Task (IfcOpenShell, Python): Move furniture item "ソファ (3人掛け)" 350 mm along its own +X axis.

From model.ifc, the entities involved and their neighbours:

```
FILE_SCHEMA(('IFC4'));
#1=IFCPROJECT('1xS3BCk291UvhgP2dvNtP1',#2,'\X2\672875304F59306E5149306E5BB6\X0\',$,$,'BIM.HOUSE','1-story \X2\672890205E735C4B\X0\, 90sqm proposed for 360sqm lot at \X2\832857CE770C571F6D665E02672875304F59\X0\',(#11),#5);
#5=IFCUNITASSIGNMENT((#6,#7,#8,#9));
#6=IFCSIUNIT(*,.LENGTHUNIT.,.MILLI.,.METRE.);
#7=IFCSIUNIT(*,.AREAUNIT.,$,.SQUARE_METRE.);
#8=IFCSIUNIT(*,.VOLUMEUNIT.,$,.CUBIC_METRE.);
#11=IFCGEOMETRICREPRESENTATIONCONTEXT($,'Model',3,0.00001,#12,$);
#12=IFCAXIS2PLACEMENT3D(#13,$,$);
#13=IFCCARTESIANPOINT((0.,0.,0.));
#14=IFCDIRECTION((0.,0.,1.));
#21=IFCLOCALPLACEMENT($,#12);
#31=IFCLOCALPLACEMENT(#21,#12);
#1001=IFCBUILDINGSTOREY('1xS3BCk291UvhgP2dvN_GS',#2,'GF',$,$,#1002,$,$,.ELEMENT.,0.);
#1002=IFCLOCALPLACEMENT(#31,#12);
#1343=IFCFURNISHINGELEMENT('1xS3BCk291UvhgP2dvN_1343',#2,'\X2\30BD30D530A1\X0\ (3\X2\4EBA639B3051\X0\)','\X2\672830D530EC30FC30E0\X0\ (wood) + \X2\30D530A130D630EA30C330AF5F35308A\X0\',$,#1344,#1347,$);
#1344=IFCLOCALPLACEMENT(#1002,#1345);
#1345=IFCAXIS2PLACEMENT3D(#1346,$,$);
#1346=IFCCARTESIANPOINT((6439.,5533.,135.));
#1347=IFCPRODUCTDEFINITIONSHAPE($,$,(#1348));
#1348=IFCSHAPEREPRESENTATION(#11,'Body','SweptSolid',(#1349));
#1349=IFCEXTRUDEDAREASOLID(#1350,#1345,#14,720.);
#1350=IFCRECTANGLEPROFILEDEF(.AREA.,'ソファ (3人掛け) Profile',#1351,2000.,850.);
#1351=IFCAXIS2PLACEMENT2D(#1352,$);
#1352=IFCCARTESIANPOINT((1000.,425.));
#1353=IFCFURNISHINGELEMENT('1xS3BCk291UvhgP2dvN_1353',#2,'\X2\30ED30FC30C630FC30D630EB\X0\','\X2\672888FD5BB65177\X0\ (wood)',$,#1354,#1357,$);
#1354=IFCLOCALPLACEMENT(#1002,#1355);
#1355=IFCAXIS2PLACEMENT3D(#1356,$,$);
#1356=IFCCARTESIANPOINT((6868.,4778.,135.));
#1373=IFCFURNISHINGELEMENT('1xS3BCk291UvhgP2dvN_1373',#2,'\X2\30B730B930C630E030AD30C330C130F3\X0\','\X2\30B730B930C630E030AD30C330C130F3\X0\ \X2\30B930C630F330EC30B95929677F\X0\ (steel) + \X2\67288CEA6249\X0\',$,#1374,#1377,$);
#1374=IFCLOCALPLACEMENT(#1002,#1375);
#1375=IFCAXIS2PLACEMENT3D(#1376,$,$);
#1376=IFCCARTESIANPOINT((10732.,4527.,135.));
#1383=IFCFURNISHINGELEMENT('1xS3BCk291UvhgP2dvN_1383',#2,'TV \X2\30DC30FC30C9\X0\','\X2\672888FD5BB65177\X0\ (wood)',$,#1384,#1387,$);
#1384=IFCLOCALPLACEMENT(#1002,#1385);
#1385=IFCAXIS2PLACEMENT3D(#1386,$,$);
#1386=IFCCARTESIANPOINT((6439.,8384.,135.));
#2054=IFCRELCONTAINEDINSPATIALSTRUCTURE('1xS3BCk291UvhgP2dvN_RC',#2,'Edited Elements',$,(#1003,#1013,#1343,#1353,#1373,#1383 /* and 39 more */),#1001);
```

```python
import ifcopenshell
import ifcopenshell.api.geometry
import ifcopenshell.util.placement

model = ifcopenshell.open("model.ifc")

item = model.by_id(1343)
matrix = ifcopenshell.util.placement.get_local_placement(item.ObjectPlacement)
matrix[:3, 3] += matrix[:3, 0] * 350.0
ifcopenshell.api.geometry.edit_object_placement(model, product=item, matrix=matrix, is_si=False)

print(ifcopenshell.util.placement.get_local_placement(item.ObjectPlacement).round(3) + 0.0)

model.write("model_updated.ifc")
```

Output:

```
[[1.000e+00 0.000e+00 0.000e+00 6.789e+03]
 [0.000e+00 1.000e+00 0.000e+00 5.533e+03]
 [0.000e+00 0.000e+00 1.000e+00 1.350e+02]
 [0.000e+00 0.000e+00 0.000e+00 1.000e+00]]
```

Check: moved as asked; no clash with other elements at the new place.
